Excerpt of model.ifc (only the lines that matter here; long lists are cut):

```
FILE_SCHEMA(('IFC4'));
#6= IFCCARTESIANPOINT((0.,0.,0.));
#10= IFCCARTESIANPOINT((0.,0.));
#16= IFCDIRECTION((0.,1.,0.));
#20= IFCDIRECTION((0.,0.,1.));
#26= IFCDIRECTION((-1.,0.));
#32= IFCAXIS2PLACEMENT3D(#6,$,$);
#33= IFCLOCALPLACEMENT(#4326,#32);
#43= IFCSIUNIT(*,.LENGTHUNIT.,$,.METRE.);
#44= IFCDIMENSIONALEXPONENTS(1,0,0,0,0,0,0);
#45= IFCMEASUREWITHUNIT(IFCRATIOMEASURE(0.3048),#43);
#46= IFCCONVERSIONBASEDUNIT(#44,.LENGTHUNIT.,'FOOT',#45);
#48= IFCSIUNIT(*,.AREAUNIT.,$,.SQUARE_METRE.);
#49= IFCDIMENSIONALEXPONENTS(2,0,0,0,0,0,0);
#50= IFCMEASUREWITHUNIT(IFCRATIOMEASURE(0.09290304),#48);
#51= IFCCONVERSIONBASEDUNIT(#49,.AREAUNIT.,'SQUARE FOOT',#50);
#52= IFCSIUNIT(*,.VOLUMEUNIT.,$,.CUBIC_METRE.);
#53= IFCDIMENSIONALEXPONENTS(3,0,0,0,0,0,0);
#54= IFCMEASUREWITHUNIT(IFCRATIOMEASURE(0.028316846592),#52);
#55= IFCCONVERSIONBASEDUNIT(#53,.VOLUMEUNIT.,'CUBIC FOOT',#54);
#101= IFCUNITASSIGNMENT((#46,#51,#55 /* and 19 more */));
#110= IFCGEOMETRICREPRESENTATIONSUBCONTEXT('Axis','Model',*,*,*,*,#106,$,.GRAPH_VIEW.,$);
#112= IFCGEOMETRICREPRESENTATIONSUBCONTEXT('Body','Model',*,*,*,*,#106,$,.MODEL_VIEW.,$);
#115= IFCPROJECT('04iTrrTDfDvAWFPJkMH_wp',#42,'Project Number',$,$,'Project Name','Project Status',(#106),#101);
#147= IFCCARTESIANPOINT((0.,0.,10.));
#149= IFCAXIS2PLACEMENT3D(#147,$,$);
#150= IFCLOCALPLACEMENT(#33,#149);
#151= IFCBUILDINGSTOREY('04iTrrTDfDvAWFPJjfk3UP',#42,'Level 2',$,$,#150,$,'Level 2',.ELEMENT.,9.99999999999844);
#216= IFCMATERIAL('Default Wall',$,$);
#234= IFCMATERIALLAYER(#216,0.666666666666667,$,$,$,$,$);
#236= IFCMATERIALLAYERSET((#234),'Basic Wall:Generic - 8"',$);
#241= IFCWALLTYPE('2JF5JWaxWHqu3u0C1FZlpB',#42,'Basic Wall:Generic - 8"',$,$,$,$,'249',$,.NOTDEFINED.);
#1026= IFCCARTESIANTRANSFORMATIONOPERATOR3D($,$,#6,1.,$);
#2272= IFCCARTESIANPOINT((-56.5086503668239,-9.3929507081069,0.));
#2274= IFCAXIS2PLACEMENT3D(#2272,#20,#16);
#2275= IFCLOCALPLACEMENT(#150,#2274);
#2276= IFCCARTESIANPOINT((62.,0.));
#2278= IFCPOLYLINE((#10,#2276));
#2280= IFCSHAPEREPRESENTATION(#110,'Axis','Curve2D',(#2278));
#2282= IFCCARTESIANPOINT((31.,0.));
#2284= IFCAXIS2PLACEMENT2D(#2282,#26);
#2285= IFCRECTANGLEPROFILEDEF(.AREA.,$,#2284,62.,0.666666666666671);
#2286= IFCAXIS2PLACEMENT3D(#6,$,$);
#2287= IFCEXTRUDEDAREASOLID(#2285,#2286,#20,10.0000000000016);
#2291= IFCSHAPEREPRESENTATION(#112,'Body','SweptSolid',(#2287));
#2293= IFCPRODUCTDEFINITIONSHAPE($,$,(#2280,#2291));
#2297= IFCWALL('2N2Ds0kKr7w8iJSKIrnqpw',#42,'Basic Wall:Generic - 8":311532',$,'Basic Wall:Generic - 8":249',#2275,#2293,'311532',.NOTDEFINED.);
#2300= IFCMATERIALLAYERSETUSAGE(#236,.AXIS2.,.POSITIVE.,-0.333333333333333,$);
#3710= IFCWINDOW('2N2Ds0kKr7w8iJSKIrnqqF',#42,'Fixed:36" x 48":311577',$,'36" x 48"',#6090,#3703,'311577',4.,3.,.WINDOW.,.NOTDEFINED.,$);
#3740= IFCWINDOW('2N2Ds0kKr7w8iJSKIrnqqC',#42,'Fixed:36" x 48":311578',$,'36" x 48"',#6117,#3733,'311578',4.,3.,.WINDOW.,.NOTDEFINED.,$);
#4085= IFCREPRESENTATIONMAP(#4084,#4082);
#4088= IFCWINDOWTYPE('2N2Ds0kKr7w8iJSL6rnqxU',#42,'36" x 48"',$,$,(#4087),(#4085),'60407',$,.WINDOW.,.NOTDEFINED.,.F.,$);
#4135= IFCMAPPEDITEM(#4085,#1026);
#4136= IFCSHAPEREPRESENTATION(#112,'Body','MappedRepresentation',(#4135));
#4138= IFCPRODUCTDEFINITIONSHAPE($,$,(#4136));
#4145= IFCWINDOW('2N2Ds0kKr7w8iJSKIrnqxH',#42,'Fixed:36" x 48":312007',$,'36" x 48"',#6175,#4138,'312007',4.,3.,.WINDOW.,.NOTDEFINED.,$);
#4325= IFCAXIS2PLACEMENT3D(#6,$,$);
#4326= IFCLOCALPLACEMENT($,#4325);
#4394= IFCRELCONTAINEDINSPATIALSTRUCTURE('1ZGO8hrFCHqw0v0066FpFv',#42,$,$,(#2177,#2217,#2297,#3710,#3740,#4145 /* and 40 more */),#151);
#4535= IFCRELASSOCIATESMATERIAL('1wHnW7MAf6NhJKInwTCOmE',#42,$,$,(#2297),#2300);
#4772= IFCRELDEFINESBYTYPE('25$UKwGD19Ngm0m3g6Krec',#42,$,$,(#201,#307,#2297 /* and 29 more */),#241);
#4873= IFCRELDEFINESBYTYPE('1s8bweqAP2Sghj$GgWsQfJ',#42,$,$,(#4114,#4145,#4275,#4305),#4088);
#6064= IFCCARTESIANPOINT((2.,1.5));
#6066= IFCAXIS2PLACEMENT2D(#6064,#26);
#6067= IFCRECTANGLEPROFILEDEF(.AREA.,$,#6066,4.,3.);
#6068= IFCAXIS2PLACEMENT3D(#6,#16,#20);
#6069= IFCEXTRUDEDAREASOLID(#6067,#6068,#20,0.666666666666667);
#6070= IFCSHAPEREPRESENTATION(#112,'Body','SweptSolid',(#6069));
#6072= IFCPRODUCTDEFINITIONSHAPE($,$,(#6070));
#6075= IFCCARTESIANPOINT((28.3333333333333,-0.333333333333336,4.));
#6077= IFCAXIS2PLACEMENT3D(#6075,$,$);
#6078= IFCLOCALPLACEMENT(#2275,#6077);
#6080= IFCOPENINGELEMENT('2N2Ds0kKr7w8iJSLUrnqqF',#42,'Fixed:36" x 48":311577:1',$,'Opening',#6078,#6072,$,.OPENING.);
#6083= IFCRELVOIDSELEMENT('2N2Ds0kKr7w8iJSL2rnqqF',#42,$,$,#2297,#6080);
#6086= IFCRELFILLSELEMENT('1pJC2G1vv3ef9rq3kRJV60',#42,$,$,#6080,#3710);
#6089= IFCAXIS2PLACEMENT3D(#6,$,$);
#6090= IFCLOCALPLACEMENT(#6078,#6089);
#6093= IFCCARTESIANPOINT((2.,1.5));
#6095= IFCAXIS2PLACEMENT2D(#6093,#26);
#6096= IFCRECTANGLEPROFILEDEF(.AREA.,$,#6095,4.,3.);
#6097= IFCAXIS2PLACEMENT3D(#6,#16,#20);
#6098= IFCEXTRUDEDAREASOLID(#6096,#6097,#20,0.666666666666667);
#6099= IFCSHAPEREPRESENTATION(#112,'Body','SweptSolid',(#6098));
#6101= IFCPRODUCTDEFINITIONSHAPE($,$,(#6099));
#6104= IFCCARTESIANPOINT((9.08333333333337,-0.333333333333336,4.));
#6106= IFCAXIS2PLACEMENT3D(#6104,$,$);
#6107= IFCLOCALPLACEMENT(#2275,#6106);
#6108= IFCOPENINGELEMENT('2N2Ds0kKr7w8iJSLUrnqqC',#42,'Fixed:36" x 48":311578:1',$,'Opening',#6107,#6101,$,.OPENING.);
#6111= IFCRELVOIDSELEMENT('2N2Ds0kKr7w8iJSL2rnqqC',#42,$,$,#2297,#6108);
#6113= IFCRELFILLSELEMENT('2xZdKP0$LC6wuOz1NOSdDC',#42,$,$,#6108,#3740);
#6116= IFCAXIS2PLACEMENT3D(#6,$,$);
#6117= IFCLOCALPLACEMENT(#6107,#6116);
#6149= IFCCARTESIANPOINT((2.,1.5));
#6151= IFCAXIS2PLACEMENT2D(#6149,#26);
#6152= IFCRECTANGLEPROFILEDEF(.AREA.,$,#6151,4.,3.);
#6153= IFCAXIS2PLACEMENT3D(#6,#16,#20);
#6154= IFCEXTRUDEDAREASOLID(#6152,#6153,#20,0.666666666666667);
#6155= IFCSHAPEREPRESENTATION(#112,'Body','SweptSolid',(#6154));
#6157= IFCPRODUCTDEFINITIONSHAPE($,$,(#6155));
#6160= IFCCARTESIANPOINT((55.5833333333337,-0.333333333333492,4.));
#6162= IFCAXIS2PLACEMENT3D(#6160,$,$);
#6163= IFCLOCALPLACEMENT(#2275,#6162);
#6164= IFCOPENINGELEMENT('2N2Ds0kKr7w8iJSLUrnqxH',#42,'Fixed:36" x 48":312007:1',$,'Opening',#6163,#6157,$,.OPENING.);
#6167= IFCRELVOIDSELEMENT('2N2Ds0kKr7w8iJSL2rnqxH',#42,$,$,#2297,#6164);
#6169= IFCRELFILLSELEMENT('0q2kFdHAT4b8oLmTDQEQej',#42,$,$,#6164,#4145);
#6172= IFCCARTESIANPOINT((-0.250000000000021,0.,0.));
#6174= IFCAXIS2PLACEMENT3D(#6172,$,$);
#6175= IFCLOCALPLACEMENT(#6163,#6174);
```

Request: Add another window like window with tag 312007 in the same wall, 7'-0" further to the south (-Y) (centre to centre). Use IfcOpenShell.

```python
import ifcopenshell
import ifcopenshell.api.feature
import ifcopenshell.api.geometry
import ifcopenshell.api.root
import ifcopenshell.geom
import ifcopenshell.util.element
import ifcopenshell.util.placement
import ifcopenshell.util.shape
import ifcopenshell.util.unit

model = ifcopenshell.open("model.ifc")
unit_scale = ifcopenshell.util.unit.calculate_unit_scale(model)
settings = ifcopenshell.geom.settings()


def volume(element):
    """Net volume in cubic metres, openings subtracted."""
    shape = ifcopenshell.geom.create_shape(settings, element)
    return ifcopenshell.util.shape.get_volume(shape.geometry)


def reuse_history(source, copy):
    """copy_class also copies each property set's owner history, people and application; keep the originals."""
    for rel in copy.IsDefinedBy:
        if rel.is_a("IfcRelDefinesByProperties") and (history := rel.RelatingPropertyDefinition.OwnerHistory):
            rel.RelatingPropertyDefinition.OwnerHistory = source.OwnerHistory
            ifcopenshell.util.element.remove_deep2(model, history)


window = model.by_id(4145)
opening = window.FillsVoids[0].RelatingOpeningElement
wall = opening.VoidsElements[0].RelatingBuildingElement
before = volume(wall)
shift = ifcopenshell.util.placement.get_local_placement(wall.ObjectPlacement)[:3, 0] * -84 * 0.0254 / unit_scale

# copy_class copies the void relationship, type, container and properties, but no geometry.
new_opening = ifcopenshell.api.root.copy_class(model, product=opening)
new_opening.Representation = ifcopenshell.util.element.copy_deep(
    model, opening.Representation, exclude=["IfcGeometricRepresentationContext", "IfcRepresentationMap"]
)
new_opening.Name = 'Fixed:36" x 48"'
new_window = ifcopenshell.api.root.copy_class(model, product=window)
new_window.Representation = ifcopenshell.util.element.copy_deep(
    model, window.Representation, exclude=["IfcGeometricRepresentationContext", "IfcRepresentationMap"]
)
new_window.Name = 'Fixed:36" x 48"'
new_window.Tag = None
reuse_history(window, new_window)
ifcopenshell.api.feature.add_filling(model, opening=new_opening, element=new_window)

for old, new in ((opening, new_opening), (window, new_window)):
    matrix = ifcopenshell.util.placement.get_local_placement(old.ObjectPlacement)
    matrix[:3, 3] += shift
    ifcopenshell.api.geometry.edit_object_placement(model, product=new, matrix=matrix, is_si=False)

after = volume(wall)

print(f"wall volume {before:.3f} -> {after:.3f} m3")

model.write("model_updated.ifc")
```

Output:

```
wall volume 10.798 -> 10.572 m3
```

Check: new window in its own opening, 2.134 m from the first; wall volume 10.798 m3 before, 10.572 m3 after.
